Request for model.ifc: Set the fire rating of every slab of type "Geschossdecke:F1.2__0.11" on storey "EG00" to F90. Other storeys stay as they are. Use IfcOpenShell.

First a look at what the model holds.

```python
import ifcopenshell
import ifcopenshell.util.element

model = ifcopenshell.open("model.ifc")
print(model.schema)
storey = next(s for s in model.by_type("IfcBuildingStorey") if s.Name == "EG00")
slabs = [e for e in ifcopenshell.util.element.get_decomposition(storey) if e.is_a("IfcSlab")]
seen = {}
for e in slabs:
    element_type = ifcopenshell.util.element.get_type(e)
    key = (element_type.Name if element_type != e and element_type else None, ifcopenshell.util.element.get_pset(e, "Pset_SlabCommon", "FireRating"))
    seen[key] = seen.get(key, 0) + 1
for (name, value), count in sorted(seen.items(), key=str):
    print(count, "x", name, "|", value)
```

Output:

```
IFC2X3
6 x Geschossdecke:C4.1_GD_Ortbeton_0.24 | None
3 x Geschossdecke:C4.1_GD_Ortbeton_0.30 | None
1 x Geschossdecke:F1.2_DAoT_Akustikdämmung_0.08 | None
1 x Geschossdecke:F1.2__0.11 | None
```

```python
import ifcopenshell
import ifcopenshell.api.pset
import ifcopenshell.util.element

model = ifcopenshell.open("model.ifc")

storey = next(s for s in model.by_type("IfcBuildingStorey") if s.Name == "EG00")
slabs = [e for e in ifcopenshell.util.element.get_decomposition(storey) if e.is_a("IfcSlab")]

count = 0
for e in slabs:
    element_type = ifcopenshell.util.element.get_type(e)
    if element_type in (None, e) or element_type.Name != "Geschossdecke:F1.2__0.11":
        continue
    # add_pset returns the element's existing set when there is one.
    pset = ifcopenshell.api.pset.add_pset(model, product=e, name="Pset_SlabCommon")
    ifcopenshell.api.pset.edit_pset(model, pset=pset, properties={"FireRating": "F90"})
    count += 1

print(count, "slabs updated")

model.write("model_v2.ifc")
```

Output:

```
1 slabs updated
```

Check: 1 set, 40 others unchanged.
